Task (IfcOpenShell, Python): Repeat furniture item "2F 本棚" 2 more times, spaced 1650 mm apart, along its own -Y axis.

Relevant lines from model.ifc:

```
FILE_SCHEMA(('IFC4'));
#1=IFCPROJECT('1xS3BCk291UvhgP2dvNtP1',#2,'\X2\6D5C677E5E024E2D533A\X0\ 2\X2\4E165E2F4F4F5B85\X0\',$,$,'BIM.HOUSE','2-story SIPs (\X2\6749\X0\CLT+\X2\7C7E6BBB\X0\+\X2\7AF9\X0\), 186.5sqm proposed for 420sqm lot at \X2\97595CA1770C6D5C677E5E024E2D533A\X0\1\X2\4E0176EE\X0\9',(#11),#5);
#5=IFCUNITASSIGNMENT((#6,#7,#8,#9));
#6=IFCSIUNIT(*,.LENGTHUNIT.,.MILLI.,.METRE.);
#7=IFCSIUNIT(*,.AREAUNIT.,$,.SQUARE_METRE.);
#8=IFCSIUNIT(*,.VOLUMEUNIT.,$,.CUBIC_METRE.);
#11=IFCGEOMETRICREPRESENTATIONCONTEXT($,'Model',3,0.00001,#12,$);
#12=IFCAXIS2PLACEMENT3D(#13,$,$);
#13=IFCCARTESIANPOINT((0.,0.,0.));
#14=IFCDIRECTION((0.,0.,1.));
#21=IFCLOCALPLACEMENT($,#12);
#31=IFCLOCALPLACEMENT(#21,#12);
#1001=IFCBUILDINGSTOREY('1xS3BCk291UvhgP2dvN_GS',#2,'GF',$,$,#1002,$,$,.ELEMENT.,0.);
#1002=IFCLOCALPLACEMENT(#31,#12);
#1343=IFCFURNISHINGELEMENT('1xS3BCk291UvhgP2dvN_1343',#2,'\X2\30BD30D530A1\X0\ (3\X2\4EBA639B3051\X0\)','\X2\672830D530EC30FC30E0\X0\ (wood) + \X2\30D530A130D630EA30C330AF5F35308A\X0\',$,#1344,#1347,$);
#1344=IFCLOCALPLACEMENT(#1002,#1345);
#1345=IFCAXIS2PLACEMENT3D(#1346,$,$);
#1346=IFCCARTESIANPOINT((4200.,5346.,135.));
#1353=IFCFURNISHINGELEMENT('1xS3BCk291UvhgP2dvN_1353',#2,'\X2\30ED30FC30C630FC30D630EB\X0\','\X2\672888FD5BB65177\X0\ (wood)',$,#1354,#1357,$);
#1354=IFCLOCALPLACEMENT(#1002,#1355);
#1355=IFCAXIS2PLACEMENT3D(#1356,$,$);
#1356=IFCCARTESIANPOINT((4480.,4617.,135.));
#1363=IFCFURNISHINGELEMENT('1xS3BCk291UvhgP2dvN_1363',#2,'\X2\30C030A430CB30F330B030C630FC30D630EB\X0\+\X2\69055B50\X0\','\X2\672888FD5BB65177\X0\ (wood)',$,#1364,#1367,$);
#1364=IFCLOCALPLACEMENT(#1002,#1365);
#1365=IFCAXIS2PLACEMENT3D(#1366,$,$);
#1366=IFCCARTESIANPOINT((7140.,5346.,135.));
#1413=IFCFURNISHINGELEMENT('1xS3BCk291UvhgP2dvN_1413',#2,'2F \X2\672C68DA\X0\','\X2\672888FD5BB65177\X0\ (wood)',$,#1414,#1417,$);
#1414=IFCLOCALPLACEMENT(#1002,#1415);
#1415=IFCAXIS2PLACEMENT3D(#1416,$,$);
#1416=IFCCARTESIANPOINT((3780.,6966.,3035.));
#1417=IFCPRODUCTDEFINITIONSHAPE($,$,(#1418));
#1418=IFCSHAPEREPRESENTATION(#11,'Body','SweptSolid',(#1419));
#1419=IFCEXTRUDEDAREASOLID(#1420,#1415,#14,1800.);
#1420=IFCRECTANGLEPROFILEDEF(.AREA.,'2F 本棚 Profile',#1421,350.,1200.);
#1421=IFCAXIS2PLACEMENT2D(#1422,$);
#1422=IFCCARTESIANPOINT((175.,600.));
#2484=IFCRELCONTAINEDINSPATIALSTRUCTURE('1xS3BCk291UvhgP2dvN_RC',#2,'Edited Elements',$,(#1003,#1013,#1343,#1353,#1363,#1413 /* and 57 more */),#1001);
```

```python
import ifcopenshell
import ifcopenshell.api.geometry
import ifcopenshell.api.root
import ifcopenshell.util.element
import ifcopenshell.util.placement

model = ifcopenshell.open("model.ifc")


def reuse_history(source, copy):
    """copy_class also copies each property set's owner history, people and application; keep the originals."""
    for rel in copy.IsDefinedBy:
        if rel.is_a("IfcRelDefinesByProperties") and (history := rel.RelatingPropertyDefinition.OwnerHistory):
            rel.RelatingPropertyDefinition.OwnerHistory = source.OwnerHistory
            ifcopenshell.util.element.remove_deep2(model, history)


source = model.by_guid("1xS3BCk291UvhgP2dvN_1413")
base = ifcopenshell.util.placement.get_local_placement(source.ObjectPlacement)
step = -base[:3, 1] * 1650.0

for i in range(1, 3):
    copy = ifcopenshell.api.root.copy_class(model, product=source)
    copy.Representation = ifcopenshell.util.element.copy_deep(
        model, source.Representation, exclude=["IfcGeometricRepresentationContext", "IfcRepresentationMap"]
    )
    reuse_history(source, copy)
    matrix = base.copy()
    matrix[:3, 3] += i * step
    print("added at", matrix[:3, 3].round(3) + 0.0)
    ifcopenshell.api.geometry.edit_object_placement(model, product=copy, matrix=matrix, is_si=False)

model.write("model-out.ifc")
```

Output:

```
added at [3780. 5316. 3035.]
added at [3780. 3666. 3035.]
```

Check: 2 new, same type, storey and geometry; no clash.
